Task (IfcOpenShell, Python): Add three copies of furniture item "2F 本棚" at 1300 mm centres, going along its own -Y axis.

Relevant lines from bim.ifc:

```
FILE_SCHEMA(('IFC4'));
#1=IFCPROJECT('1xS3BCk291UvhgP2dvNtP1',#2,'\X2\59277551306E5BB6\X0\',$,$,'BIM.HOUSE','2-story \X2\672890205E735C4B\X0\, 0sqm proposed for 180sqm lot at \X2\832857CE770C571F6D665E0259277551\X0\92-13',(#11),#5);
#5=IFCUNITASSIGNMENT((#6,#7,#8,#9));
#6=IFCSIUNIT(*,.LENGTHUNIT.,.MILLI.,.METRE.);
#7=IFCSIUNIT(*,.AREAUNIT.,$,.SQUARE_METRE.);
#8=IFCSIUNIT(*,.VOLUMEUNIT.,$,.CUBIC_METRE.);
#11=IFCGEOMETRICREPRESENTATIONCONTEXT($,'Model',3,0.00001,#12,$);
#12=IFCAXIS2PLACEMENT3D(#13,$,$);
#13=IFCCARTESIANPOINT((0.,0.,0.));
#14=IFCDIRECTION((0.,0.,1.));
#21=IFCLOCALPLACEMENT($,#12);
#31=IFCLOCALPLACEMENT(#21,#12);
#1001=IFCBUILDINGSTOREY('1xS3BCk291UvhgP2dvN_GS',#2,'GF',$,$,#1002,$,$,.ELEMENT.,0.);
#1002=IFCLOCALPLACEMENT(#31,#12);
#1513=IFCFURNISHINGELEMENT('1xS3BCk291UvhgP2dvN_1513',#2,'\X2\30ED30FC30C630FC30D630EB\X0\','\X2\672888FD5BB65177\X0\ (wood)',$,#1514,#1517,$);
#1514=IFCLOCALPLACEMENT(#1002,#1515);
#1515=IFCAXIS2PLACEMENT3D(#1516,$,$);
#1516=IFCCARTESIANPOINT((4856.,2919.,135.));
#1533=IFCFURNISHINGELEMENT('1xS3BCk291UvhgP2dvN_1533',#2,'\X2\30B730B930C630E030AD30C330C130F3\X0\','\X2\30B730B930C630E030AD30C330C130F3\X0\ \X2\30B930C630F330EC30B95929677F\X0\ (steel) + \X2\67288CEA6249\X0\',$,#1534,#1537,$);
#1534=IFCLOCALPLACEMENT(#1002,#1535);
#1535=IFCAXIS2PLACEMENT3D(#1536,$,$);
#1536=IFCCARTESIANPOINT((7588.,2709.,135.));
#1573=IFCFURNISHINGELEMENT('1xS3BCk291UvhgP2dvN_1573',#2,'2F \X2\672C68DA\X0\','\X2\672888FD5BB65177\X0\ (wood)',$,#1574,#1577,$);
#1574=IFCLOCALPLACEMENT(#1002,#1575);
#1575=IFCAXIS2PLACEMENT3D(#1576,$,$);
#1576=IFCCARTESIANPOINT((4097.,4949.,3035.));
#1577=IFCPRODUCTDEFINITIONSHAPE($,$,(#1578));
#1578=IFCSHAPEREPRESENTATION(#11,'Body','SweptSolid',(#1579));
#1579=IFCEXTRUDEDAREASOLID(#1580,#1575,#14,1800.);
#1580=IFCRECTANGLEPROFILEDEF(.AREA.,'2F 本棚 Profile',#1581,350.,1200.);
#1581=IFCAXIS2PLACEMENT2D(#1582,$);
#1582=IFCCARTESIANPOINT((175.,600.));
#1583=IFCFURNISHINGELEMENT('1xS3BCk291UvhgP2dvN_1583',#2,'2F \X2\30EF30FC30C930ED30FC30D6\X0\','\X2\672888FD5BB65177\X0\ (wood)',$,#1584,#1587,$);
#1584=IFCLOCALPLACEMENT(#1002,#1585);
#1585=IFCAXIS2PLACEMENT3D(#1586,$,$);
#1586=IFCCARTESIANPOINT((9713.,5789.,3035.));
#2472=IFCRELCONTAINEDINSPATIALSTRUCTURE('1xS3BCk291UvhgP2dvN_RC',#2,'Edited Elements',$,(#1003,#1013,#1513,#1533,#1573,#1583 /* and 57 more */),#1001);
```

```python
import ifcopenshell
import ifcopenshell.api.geometry
import ifcopenshell.api.root
import ifcopenshell.util.element
import ifcopenshell.util.placement

model = ifcopenshell.open("bim.ifc")


def reuse_history(source, copy):
    """copy_class also copies each property set's owner history, people and application; keep the originals."""
    for rel in copy.IsDefinedBy:
        if rel.is_a("IfcRelDefinesByProperties") and (history := rel.RelatingPropertyDefinition.OwnerHistory):
            rel.RelatingPropertyDefinition.OwnerHistory = source.OwnerHistory
            ifcopenshell.util.element.remove_deep2(model, history)


source = model.by_guid("1xS3BCk291UvhgP2dvN_1573")
base = ifcopenshell.util.placement.get_local_placement(source.ObjectPlacement)
step = -base[:3, 1] * 1300.0

for i in range(1, 4):
    copy = ifcopenshell.api.root.copy_class(model, product=source)
    copy.Representation = ifcopenshell.util.element.copy_deep(
        model, source.Representation, exclude=["IfcGeometricRepresentationContext", "IfcRepresentationMap"]
    )
    reuse_history(source, copy)
    matrix = base.copy()
    matrix[:3, 3] += i * step
    print("added at", matrix[:3, 3].round(3) + 0.0)
    ifcopenshell.api.geometry.edit_object_placement(model, product=copy, matrix=matrix, is_si=False)

model.write("bim_updated.ifc")
```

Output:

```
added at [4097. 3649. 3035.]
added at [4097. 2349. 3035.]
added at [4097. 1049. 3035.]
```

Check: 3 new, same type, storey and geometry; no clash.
